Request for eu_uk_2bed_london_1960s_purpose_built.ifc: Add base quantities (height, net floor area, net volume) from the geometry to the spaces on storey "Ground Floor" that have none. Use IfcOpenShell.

First a look at what the model holds.

```python
import ifcopenshell
import ifcopenshell.util.element
import ifcopenshell.util.unit

model = ifcopenshell.open("eu_uk_2bed_london_1960s_purpose_built.ifc")
print(model.schema)
for unit_type in ("LENGTHUNIT", "AREAUNIT", "VOLUMEUNIT"):
    print(unit_type, ifcopenshell.util.unit.calculate_unit_scale(model, unit_type))
storey = next(s for s in model.by_type("IfcBuildingStorey") if s.Name == "Ground Floor")
spaces = [e for e in ifcopenshell.util.element.get_decomposition(storey) if e.is_a("IfcSpace")]
for e in sorted(spaces, key=lambda e: e.id()):
    print(e.id(), e.is_a(), e.Name, list(ifcopenshell.util.element.get_psets(e, qtos_only=True)), sep=" | ")
```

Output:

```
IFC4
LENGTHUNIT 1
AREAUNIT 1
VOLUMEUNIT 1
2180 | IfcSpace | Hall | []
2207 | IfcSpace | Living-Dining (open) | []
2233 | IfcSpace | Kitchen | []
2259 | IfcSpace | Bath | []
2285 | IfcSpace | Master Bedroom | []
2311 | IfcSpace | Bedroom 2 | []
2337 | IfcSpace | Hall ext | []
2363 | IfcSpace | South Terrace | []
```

```python
import ifcopenshell
import ifcopenshell.api.pset
import ifcopenshell.geom
import ifcopenshell.util.element
import ifcopenshell.util.shape
import ifcopenshell.util.unit

model = ifcopenshell.open("eu_uk_2bed_london_1960s_purpose_built.ifc")
unit_scale = ifcopenshell.util.unit.calculate_unit_scale(model)
area_scale = ifcopenshell.util.unit.calculate_unit_scale(model, "AREAUNIT")
volume_scale = ifcopenshell.util.unit.calculate_unit_scale(model, "VOLUMEUNIT")
settings = ifcopenshell.geom.settings()

storey = next(s for s in model.by_type("IfcBuildingStorey") if s.Name == "Ground Floor")
spaces = [e for e in ifcopenshell.util.element.get_decomposition(storey) if e.is_a("IfcSpace")]

for e in sorted(spaces, key=lambda e: e.id()):
    if ifcopenshell.util.element.get_psets(e, qtos_only=True, should_inherit=False):
        continue
    # Geometry comes back in metres, in the element's own axes.
    shape = ifcopenshell.geom.create_shape(settings, e)
    values = {
        "Height": ifcopenshell.util.shape.get_z(shape.geometry) / unit_scale,
        "NetFloorArea": ifcopenshell.util.shape.get_footprint_area(shape.geometry) / area_scale,
        "NetVolume": ifcopenshell.util.shape.get_volume(shape.geometry) / volume_scale,
    }
    qto = ifcopenshell.api.pset.add_qto(model, product=e, name="Qto_SpaceBaseQuantities")
    ifcopenshell.api.pset.edit_qto(model, qto=qto, properties=values)
    print(e.id(), {k: round(v, 3) for k, v in values.items()})

model.write("eu_uk_2bed_london_1960s_purpose_built_v2.ifc")
```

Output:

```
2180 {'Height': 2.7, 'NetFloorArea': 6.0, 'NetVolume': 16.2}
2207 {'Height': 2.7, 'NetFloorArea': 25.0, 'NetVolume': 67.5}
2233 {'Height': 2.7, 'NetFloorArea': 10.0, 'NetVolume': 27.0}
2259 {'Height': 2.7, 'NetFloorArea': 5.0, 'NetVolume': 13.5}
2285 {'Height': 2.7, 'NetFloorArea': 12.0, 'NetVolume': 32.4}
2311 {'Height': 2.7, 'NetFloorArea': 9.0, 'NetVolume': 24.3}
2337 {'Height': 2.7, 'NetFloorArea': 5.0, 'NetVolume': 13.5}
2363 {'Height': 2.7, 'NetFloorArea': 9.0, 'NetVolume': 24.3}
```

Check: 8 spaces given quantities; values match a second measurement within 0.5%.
